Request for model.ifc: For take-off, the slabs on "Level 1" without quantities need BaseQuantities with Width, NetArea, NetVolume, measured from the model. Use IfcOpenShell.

First a look at what the model holds.

```python
import ifcopenshell
import ifcopenshell.util.element
import ifcopenshell.util.unit

model = ifcopenshell.open("model.ifc")
print(model.schema)
for unit_type in ("LENGTHUNIT", "AREAUNIT", "VOLUMEUNIT"):
    print(unit_type, ifcopenshell.util.unit.calculate_unit_scale(model, unit_type))
storey = next(s for s in model.by_type("IfcBuildingStorey") if s.Name == "Level 1")
slabs = [e for e in ifcopenshell.util.element.get_decomposition(storey) if e.is_a("IfcSlab")]
for e in sorted(slabs, key=lambda e: e.id()):
    print(e.id(), e.is_a(), e.Name, list(ifcopenshell.util.element.get_psets(e, qtos_only=True)), sep=" | ")
```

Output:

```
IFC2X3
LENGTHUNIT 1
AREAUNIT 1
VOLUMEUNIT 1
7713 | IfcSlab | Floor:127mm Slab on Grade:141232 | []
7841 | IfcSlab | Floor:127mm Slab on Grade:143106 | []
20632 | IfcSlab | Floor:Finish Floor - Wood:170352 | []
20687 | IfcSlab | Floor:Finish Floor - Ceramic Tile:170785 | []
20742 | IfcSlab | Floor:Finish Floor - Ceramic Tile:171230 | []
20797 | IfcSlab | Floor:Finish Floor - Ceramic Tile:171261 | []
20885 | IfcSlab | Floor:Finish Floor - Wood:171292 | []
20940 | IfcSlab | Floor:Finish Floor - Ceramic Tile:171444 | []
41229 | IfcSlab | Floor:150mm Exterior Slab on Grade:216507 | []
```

```python
import ifcopenshell
import ifcopenshell.api.pset
import ifcopenshell.geom
import ifcopenshell.util.element
import ifcopenshell.util.shape
import ifcopenshell.util.unit

model = ifcopenshell.open("model.ifc")
unit_scale = ifcopenshell.util.unit.calculate_unit_scale(model)
area_scale = ifcopenshell.util.unit.calculate_unit_scale(model, "AREAUNIT")
volume_scale = ifcopenshell.util.unit.calculate_unit_scale(model, "VOLUMEUNIT")
settings = ifcopenshell.geom.settings()

storey = next(s for s in model.by_type("IfcBuildingStorey") if s.Name == "Level 1")
slabs = [e for e in ifcopenshell.util.element.get_decomposition(storey) if e.is_a("IfcSlab")]

for e in sorted(slabs, key=lambda e: e.id()):
    if ifcopenshell.util.element.get_psets(e, qtos_only=True, should_inherit=False):
        continue
    # Geometry comes back in metres, in the element's own axes.
    shape = ifcopenshell.geom.create_shape(settings, e)
    values = {
        "Width": ifcopenshell.util.shape.get_z(shape.geometry) / unit_scale,
        "NetArea": ifcopenshell.util.shape.get_footprint_area(shape.geometry) / area_scale,
        "NetVolume": ifcopenshell.util.shape.get_volume(shape.geometry) / volume_scale,
    }
    qto = ifcopenshell.api.pset.add_qto(model, product=e, name="BaseQuantities")
    ifcopenshell.api.pset.edit_qto(model, qto=qto, properties=values)
    print(e.id(), {k: round(v, 3) for k, v in values.items()})

model.write("model_updated.ifc")
```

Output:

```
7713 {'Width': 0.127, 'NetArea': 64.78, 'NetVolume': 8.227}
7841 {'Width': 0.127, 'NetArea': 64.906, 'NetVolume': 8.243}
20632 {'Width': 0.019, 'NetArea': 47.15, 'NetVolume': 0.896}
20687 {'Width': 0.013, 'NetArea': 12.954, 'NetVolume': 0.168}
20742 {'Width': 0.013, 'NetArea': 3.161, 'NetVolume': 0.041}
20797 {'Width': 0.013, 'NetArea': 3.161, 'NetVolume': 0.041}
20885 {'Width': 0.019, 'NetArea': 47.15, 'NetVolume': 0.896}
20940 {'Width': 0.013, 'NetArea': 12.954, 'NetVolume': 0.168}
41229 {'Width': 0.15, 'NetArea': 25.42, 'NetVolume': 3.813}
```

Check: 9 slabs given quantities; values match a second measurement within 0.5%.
